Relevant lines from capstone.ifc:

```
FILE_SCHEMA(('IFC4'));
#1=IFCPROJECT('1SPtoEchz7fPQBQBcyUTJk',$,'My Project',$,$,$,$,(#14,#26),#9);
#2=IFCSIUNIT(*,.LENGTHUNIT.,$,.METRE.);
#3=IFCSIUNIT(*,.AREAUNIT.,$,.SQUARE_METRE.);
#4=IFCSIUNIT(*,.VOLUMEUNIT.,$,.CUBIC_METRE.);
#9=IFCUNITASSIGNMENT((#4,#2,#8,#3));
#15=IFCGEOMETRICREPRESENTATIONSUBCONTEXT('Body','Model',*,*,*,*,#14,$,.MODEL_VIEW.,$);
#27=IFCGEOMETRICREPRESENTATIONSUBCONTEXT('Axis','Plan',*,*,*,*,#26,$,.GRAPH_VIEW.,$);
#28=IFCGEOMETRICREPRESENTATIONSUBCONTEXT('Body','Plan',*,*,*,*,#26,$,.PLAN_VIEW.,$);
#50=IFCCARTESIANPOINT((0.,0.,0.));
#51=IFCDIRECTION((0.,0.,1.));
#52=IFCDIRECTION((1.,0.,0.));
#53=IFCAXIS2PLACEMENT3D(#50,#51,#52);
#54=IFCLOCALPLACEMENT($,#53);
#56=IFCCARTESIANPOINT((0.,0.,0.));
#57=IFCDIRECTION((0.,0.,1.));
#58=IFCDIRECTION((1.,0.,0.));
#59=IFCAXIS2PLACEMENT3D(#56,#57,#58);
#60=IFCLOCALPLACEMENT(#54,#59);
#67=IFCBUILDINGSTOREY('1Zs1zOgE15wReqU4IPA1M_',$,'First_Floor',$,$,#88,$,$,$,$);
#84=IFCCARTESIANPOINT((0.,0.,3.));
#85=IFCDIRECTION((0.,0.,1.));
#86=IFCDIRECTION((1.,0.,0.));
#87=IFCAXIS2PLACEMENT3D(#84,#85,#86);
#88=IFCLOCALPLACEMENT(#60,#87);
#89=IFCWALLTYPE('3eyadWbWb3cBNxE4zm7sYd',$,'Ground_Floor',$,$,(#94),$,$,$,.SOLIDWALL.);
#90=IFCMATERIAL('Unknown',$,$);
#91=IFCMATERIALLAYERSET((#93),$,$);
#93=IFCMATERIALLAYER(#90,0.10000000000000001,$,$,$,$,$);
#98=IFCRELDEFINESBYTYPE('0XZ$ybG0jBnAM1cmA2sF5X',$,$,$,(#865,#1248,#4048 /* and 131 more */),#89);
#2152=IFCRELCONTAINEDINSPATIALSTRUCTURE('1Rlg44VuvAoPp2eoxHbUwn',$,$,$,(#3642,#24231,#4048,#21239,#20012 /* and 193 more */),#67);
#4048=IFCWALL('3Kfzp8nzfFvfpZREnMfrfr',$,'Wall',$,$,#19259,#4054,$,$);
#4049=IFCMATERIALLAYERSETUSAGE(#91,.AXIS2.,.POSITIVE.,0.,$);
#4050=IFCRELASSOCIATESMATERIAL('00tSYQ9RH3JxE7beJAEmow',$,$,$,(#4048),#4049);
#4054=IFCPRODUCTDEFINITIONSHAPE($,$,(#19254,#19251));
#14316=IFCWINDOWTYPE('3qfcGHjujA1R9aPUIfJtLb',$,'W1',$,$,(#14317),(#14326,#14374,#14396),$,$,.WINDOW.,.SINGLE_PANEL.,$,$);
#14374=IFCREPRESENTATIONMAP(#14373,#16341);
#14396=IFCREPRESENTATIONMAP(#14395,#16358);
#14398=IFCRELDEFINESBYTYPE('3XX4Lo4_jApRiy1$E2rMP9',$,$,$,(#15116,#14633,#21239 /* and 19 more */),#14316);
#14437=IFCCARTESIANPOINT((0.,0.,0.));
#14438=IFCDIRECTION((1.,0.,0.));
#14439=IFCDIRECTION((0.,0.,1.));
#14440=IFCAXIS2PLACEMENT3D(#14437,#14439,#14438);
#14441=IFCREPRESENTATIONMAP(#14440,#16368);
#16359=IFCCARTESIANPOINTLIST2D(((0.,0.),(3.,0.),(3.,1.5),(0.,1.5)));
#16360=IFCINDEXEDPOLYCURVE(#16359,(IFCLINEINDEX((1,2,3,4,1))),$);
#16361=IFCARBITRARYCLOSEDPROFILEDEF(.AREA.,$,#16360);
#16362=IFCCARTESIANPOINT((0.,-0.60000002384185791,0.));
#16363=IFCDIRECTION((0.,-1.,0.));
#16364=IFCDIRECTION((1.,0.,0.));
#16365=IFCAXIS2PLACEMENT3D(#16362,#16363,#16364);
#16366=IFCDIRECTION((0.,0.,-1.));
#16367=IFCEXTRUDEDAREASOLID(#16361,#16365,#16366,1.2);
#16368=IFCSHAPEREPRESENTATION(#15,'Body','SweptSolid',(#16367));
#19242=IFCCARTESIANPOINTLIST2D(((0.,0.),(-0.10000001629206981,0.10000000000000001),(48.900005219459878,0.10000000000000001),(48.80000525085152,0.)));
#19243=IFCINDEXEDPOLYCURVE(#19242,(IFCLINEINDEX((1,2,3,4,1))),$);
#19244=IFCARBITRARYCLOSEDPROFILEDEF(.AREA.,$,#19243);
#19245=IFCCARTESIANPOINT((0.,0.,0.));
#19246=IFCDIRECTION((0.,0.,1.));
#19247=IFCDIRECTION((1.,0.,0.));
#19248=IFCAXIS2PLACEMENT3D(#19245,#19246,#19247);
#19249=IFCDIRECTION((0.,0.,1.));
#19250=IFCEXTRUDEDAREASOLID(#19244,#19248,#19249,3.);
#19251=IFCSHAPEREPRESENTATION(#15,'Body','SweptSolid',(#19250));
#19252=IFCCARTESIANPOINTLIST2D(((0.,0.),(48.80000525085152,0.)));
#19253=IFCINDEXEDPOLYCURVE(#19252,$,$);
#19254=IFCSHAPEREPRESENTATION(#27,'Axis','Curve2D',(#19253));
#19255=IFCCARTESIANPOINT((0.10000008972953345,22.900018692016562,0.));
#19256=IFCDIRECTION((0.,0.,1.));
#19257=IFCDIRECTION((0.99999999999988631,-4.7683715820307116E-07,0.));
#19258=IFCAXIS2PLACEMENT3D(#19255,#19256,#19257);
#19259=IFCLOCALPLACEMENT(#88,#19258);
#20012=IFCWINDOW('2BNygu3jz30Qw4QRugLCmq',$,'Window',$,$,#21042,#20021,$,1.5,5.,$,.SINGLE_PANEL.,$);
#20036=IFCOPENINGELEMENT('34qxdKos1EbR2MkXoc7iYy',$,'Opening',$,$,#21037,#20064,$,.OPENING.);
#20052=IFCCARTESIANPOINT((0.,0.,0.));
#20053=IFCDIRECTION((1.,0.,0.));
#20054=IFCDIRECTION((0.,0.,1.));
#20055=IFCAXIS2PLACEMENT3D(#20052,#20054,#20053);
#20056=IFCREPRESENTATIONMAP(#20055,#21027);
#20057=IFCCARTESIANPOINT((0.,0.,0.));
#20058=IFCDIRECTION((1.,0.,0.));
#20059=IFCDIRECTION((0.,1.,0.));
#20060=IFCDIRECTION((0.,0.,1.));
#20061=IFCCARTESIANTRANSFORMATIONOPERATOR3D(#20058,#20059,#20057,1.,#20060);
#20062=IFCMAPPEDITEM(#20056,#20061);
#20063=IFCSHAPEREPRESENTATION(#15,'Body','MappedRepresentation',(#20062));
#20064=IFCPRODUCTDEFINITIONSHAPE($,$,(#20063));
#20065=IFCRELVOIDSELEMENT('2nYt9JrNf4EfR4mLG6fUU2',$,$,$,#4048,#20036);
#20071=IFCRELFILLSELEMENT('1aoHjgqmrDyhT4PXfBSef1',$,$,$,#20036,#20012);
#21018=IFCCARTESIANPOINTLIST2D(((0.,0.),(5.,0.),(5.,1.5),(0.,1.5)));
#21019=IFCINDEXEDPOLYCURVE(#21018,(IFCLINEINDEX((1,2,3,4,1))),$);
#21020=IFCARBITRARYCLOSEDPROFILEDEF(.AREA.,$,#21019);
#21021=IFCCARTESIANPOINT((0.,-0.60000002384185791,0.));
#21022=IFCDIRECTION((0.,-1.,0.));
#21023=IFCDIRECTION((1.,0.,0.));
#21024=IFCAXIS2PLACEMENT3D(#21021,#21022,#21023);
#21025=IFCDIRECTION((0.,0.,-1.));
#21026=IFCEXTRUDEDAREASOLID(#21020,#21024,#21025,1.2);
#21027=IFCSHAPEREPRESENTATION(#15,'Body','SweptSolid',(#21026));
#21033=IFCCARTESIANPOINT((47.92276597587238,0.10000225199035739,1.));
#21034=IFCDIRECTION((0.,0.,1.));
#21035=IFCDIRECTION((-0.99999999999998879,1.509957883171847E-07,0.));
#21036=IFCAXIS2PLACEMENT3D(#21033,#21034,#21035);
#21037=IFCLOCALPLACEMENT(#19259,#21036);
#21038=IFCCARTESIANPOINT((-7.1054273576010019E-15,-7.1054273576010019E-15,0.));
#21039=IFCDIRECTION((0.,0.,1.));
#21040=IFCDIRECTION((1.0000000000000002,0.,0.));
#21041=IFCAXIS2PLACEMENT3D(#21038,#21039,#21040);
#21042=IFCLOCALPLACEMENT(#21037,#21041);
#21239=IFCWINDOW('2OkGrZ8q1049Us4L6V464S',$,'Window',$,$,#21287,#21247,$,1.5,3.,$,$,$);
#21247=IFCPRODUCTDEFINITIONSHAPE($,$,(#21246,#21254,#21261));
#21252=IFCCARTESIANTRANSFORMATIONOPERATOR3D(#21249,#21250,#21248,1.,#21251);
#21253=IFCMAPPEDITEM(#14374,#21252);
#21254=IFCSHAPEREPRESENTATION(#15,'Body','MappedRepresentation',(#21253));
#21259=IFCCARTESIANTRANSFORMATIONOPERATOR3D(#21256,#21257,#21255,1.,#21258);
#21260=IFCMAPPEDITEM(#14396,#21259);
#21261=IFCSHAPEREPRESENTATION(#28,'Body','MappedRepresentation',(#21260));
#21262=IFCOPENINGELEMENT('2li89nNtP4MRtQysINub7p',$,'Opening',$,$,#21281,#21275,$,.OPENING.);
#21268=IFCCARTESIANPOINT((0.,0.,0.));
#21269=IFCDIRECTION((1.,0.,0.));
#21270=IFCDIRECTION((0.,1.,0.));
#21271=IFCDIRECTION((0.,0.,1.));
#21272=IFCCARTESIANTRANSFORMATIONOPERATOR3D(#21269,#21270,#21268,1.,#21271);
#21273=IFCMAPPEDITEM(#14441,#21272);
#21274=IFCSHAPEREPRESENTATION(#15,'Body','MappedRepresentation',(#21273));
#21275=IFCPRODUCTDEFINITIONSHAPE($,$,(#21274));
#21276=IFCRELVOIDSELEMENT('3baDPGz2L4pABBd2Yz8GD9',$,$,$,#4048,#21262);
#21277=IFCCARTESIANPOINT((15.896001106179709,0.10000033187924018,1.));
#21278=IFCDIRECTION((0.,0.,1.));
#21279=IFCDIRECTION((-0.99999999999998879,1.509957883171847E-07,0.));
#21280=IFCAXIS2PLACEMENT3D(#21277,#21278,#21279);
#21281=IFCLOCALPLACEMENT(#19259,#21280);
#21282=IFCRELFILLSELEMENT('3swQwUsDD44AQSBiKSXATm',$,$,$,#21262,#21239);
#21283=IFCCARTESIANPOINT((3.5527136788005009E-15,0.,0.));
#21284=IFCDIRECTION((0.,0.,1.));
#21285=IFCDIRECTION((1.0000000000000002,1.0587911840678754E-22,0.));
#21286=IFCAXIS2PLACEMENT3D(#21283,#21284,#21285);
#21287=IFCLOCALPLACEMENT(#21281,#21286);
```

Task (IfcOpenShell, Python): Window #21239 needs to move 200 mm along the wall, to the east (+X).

```python
import ifcopenshell
import ifcopenshell.api.geometry
import ifcopenshell.util.placement
import ifcopenshell.util.unit

model = ifcopenshell.open("capstone.ifc")
unit_scale = ifcopenshell.util.unit.calculate_unit_scale(model)

window = model.by_guid("2OkGrZ8q1049Us4L6V464S")
opening = window.FillsVoids[0].RelatingOpeningElement
wall = opening.VoidsElements[0].RelatingBuildingElement

wall_matrix = ifcopenshell.util.placement.get_local_placement(wall.ObjectPlacement)
shift = wall_matrix[:3, 0] * 0.2 / unit_scale
before = ifcopenshell.util.placement.get_local_placement(window.ObjectPlacement)[:3, 3].copy()

# The window is placed relative to its opening, so it follows when the opening moves.
matrix = ifcopenshell.util.placement.get_local_placement(opening.ObjectPlacement)
matrix[:3, 3] += shift
ifcopenshell.api.geometry.edit_object_placement(
    model, product=opening, matrix=matrix, is_si=False, should_transform_children=True
)

after = ifcopenshell.util.placement.get_local_placement(window.ObjectPlacement)[:3, 3]
print("window moved by", (after - before).round(3) + 0.0)

model.write("capstone_rev.ifc")
```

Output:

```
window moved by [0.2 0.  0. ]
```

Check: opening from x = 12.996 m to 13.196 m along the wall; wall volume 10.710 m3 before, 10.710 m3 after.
